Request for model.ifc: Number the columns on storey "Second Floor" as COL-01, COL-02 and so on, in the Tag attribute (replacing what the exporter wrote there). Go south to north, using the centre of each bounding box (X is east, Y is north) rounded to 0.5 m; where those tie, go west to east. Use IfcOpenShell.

First a look at what the model holds.

```python
import ifcopenshell
import ifcopenshell.util.element
import ifcopenshell.util.placement

model = ifcopenshell.open("model.ifc")
print(model.schema)
storey = next(s for s in model.by_type("IfcBuildingStorey") if s.Name == "Second Floor")
columns = [e for e in ifcopenshell.util.element.get_decomposition(storey) if e.is_a("IfcColumn")]
for e in sorted(columns, key=lambda e: e.id()):
    origin = ifcopenshell.util.placement.get_local_placement(e.ObjectPlacement)[:3, 3]
    print(e.id(), e.Tag, e.Name, origin.round(2) + 0.0, sep=" | ")
```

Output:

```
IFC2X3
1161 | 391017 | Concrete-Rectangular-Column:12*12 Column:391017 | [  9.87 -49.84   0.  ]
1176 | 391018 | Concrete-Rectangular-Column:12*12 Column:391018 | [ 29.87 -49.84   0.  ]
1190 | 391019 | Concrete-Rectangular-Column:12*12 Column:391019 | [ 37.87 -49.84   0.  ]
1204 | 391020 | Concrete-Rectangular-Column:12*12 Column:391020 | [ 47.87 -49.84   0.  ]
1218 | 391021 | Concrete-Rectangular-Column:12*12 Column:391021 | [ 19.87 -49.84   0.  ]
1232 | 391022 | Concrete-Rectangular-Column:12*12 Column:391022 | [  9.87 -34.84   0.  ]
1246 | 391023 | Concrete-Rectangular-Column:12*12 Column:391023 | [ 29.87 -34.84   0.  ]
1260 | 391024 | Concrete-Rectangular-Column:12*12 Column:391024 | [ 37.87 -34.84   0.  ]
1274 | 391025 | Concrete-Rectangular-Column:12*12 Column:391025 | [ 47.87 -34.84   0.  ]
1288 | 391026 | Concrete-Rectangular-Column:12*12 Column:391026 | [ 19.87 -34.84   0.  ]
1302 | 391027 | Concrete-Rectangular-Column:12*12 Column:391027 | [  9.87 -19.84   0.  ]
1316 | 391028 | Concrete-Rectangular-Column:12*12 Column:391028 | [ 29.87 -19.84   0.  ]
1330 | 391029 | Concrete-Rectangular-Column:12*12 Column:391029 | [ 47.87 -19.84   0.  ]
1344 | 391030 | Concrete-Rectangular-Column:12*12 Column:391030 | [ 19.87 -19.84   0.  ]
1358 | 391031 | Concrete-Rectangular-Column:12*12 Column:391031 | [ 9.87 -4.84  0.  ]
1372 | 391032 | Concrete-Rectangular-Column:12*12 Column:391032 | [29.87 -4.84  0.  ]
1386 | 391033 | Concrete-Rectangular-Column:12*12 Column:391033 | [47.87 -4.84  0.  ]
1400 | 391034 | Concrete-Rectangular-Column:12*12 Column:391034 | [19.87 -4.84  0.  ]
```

```python
import ifcopenshell
import ifcopenshell.geom
import ifcopenshell.util.element
import ifcopenshell.util.shape

model = ifcopenshell.open("model.ifc")
settings = ifcopenshell.geom.settings()
settings.set("use-world-coords", True)


def centre(element):
    shape = ifcopenshell.geom.create_shape(settings, element)
    return ifcopenshell.util.shape.get_bbox_centroid(shape.geometry)


storey = next(s for s in model.by_type("IfcBuildingStorey") if s.Name == "Second Floor")
columns = [e for e in ifcopenshell.util.element.get_decomposition(storey) if e.is_a("IfcColumn")]

# Insertion points can sit at a corner or the storey origin, so sort by the geometry (in metres).
centres = {e: centre(e) for e in columns}
columns.sort(key=lambda e: (round(centres[e][1] / 0.5), centres[e][0]))

for i, e in enumerate(columns, start=1):
    number = f"COL-{i:02d}"
    e.Tag = number
    print(e.id(), number)

model.write("model-out.ifc")
```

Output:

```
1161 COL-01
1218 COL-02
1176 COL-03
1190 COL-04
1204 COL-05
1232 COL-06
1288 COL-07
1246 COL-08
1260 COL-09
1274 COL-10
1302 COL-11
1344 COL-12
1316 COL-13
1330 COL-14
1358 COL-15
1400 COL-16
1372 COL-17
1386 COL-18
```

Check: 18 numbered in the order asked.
